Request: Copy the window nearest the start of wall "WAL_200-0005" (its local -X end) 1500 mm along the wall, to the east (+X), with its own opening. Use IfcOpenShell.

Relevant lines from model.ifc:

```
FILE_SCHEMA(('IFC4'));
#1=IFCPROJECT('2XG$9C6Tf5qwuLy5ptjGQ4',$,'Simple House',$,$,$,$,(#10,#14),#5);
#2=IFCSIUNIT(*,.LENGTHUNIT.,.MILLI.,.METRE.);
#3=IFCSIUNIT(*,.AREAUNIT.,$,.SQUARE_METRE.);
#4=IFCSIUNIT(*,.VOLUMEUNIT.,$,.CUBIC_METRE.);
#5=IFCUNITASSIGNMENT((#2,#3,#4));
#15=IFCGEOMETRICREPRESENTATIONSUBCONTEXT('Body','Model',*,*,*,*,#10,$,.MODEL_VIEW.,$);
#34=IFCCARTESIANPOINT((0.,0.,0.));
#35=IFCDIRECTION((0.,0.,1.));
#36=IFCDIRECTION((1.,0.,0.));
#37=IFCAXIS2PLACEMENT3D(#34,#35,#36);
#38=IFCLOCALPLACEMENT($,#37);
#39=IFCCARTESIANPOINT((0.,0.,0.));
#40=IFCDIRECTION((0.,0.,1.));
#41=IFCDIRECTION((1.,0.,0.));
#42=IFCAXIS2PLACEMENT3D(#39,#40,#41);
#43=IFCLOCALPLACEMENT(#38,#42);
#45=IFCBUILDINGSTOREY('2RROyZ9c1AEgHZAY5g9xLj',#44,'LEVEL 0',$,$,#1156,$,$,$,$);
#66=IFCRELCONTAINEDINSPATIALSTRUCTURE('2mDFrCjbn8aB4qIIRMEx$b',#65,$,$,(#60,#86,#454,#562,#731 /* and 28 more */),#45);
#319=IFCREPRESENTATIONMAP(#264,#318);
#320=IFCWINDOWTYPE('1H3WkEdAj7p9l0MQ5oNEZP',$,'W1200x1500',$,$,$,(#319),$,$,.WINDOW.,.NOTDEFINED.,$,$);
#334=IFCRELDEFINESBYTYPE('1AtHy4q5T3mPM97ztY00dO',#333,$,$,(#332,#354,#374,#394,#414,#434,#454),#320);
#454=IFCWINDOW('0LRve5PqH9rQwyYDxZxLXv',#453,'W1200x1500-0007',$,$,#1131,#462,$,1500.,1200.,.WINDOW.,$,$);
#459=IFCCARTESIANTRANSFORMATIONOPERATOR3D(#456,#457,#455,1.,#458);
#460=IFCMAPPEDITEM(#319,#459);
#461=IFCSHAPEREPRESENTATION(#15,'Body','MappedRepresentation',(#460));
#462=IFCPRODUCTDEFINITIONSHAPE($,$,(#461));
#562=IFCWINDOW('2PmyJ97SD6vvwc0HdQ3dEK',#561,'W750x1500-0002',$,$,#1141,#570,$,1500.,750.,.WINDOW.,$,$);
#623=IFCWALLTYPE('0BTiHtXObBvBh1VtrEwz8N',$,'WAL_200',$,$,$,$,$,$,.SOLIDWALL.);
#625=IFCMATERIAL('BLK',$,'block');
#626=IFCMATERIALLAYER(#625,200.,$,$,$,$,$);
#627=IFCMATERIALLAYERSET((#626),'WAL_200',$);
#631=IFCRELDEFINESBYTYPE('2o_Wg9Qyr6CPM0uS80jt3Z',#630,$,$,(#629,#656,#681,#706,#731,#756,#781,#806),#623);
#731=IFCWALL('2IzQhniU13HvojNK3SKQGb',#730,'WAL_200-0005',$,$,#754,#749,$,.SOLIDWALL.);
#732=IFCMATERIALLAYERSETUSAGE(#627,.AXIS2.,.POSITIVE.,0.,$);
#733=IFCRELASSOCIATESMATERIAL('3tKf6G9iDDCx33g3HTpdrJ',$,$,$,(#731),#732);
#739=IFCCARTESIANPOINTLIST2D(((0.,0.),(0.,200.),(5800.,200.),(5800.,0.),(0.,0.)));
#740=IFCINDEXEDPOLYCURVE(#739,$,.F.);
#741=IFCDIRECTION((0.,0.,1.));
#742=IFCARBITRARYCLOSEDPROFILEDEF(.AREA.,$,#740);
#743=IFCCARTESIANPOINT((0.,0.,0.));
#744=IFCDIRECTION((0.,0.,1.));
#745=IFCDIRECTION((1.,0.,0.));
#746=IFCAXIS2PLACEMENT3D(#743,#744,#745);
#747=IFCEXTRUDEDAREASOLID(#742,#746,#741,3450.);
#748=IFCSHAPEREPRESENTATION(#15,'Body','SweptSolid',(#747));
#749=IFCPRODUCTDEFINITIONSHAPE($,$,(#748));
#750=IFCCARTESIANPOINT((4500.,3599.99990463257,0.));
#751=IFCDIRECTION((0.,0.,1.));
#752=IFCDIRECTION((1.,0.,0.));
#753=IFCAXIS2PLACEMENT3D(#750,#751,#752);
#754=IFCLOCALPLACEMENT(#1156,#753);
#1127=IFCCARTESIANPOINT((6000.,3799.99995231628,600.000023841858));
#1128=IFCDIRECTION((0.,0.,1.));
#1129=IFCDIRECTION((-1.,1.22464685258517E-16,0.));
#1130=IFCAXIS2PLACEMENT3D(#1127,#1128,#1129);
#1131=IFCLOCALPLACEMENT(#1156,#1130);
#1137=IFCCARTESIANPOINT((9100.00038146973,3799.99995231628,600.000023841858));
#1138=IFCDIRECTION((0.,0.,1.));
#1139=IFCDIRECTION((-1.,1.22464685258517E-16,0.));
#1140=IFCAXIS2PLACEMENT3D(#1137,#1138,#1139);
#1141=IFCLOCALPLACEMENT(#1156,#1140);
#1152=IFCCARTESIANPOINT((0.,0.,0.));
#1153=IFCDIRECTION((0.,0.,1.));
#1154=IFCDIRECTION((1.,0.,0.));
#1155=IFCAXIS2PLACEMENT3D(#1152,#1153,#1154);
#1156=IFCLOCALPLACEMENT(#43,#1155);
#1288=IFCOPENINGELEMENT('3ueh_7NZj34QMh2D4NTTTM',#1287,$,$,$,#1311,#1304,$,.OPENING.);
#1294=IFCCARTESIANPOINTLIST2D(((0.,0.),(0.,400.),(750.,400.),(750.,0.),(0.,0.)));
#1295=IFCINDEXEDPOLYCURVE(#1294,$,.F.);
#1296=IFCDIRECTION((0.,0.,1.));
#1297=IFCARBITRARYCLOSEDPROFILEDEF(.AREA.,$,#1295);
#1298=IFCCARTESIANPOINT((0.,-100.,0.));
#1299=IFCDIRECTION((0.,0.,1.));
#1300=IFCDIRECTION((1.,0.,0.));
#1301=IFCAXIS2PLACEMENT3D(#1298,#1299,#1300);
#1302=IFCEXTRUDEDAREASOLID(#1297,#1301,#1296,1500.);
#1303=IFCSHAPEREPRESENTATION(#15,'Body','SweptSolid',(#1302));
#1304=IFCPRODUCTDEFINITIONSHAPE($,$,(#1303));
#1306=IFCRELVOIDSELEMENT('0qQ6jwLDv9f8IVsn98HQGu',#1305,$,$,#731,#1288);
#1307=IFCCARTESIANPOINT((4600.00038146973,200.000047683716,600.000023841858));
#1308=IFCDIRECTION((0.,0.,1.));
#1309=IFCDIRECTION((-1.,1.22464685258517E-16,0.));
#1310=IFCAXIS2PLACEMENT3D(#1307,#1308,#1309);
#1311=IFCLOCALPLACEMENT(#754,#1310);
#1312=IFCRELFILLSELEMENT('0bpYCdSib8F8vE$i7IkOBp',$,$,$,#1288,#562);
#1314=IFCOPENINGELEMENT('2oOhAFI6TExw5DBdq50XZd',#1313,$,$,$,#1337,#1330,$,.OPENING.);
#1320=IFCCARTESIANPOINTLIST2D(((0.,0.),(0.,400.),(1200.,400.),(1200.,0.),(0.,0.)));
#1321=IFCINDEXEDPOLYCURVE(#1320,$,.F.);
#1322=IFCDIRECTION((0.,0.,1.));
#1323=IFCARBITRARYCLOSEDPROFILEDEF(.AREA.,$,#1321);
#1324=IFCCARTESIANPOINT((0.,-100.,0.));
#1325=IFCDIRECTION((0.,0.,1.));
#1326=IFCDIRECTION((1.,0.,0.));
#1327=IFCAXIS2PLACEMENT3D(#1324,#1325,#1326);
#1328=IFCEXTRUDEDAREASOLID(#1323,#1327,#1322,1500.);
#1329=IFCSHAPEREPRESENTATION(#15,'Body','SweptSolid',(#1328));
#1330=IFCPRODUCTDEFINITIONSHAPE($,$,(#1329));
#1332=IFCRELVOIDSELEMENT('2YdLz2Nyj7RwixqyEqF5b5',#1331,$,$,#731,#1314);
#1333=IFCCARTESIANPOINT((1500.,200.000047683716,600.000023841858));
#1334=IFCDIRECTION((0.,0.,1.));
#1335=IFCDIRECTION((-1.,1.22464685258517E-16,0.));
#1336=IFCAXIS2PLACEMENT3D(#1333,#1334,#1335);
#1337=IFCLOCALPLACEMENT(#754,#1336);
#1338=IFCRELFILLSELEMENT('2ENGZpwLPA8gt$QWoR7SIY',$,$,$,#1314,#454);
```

```python
import ifcopenshell
import ifcopenshell.api.feature
import ifcopenshell.api.geometry
import ifcopenshell.api.root
import ifcopenshell.geom
import ifcopenshell.util.element
import ifcopenshell.util.placement
import ifcopenshell.util.shape
import ifcopenshell.util.unit

model = ifcopenshell.open("model.ifc")
unit_scale = ifcopenshell.util.unit.calculate_unit_scale(model)
settings = ifcopenshell.geom.settings()


def volume(element):
    """Net volume in cubic metres, openings subtracted."""
    shape = ifcopenshell.geom.create_shape(settings, element)
    return ifcopenshell.util.shape.get_volume(shape.geometry)


window = model.by_guid("0LRve5PqH9rQwyYDxZxLXv")
opening = window.FillsVoids[0].RelatingOpeningElement
wall = opening.VoidsElements[0].RelatingBuildingElement
before = volume(wall)
shift = ifcopenshell.util.placement.get_local_placement(wall.ObjectPlacement)[:3, 0] * 1.5 / unit_scale

# copy_class copies the void relationship, type, container and properties, but no geometry.
new_opening = ifcopenshell.api.root.copy_class(model, product=opening)
new_opening.Representation = ifcopenshell.util.element.copy_deep(
    model, opening.Representation, exclude=["IfcGeometricRepresentationContext", "IfcRepresentationMap"]
)
new_window = ifcopenshell.api.root.copy_class(model, product=window)
new_window.Representation = ifcopenshell.util.element.copy_deep(
    model, window.Representation, exclude=["IfcGeometricRepresentationContext", "IfcRepresentationMap"]
)
ifcopenshell.api.feature.add_filling(model, opening=new_opening, element=new_window)

for old, new in ((opening, new_opening), (window, new_window)):
    matrix = ifcopenshell.util.placement.get_local_placement(old.ObjectPlacement)
    matrix[:3, 3] += shift
    ifcopenshell.api.geometry.edit_object_placement(model, product=new, matrix=matrix, is_si=False)

after = volume(wall)

print(f"wall volume {before:.3f} -> {after:.3f} m3")

model.write("model_rev.ifc")
```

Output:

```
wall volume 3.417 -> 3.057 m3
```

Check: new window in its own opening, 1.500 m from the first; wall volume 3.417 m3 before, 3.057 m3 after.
